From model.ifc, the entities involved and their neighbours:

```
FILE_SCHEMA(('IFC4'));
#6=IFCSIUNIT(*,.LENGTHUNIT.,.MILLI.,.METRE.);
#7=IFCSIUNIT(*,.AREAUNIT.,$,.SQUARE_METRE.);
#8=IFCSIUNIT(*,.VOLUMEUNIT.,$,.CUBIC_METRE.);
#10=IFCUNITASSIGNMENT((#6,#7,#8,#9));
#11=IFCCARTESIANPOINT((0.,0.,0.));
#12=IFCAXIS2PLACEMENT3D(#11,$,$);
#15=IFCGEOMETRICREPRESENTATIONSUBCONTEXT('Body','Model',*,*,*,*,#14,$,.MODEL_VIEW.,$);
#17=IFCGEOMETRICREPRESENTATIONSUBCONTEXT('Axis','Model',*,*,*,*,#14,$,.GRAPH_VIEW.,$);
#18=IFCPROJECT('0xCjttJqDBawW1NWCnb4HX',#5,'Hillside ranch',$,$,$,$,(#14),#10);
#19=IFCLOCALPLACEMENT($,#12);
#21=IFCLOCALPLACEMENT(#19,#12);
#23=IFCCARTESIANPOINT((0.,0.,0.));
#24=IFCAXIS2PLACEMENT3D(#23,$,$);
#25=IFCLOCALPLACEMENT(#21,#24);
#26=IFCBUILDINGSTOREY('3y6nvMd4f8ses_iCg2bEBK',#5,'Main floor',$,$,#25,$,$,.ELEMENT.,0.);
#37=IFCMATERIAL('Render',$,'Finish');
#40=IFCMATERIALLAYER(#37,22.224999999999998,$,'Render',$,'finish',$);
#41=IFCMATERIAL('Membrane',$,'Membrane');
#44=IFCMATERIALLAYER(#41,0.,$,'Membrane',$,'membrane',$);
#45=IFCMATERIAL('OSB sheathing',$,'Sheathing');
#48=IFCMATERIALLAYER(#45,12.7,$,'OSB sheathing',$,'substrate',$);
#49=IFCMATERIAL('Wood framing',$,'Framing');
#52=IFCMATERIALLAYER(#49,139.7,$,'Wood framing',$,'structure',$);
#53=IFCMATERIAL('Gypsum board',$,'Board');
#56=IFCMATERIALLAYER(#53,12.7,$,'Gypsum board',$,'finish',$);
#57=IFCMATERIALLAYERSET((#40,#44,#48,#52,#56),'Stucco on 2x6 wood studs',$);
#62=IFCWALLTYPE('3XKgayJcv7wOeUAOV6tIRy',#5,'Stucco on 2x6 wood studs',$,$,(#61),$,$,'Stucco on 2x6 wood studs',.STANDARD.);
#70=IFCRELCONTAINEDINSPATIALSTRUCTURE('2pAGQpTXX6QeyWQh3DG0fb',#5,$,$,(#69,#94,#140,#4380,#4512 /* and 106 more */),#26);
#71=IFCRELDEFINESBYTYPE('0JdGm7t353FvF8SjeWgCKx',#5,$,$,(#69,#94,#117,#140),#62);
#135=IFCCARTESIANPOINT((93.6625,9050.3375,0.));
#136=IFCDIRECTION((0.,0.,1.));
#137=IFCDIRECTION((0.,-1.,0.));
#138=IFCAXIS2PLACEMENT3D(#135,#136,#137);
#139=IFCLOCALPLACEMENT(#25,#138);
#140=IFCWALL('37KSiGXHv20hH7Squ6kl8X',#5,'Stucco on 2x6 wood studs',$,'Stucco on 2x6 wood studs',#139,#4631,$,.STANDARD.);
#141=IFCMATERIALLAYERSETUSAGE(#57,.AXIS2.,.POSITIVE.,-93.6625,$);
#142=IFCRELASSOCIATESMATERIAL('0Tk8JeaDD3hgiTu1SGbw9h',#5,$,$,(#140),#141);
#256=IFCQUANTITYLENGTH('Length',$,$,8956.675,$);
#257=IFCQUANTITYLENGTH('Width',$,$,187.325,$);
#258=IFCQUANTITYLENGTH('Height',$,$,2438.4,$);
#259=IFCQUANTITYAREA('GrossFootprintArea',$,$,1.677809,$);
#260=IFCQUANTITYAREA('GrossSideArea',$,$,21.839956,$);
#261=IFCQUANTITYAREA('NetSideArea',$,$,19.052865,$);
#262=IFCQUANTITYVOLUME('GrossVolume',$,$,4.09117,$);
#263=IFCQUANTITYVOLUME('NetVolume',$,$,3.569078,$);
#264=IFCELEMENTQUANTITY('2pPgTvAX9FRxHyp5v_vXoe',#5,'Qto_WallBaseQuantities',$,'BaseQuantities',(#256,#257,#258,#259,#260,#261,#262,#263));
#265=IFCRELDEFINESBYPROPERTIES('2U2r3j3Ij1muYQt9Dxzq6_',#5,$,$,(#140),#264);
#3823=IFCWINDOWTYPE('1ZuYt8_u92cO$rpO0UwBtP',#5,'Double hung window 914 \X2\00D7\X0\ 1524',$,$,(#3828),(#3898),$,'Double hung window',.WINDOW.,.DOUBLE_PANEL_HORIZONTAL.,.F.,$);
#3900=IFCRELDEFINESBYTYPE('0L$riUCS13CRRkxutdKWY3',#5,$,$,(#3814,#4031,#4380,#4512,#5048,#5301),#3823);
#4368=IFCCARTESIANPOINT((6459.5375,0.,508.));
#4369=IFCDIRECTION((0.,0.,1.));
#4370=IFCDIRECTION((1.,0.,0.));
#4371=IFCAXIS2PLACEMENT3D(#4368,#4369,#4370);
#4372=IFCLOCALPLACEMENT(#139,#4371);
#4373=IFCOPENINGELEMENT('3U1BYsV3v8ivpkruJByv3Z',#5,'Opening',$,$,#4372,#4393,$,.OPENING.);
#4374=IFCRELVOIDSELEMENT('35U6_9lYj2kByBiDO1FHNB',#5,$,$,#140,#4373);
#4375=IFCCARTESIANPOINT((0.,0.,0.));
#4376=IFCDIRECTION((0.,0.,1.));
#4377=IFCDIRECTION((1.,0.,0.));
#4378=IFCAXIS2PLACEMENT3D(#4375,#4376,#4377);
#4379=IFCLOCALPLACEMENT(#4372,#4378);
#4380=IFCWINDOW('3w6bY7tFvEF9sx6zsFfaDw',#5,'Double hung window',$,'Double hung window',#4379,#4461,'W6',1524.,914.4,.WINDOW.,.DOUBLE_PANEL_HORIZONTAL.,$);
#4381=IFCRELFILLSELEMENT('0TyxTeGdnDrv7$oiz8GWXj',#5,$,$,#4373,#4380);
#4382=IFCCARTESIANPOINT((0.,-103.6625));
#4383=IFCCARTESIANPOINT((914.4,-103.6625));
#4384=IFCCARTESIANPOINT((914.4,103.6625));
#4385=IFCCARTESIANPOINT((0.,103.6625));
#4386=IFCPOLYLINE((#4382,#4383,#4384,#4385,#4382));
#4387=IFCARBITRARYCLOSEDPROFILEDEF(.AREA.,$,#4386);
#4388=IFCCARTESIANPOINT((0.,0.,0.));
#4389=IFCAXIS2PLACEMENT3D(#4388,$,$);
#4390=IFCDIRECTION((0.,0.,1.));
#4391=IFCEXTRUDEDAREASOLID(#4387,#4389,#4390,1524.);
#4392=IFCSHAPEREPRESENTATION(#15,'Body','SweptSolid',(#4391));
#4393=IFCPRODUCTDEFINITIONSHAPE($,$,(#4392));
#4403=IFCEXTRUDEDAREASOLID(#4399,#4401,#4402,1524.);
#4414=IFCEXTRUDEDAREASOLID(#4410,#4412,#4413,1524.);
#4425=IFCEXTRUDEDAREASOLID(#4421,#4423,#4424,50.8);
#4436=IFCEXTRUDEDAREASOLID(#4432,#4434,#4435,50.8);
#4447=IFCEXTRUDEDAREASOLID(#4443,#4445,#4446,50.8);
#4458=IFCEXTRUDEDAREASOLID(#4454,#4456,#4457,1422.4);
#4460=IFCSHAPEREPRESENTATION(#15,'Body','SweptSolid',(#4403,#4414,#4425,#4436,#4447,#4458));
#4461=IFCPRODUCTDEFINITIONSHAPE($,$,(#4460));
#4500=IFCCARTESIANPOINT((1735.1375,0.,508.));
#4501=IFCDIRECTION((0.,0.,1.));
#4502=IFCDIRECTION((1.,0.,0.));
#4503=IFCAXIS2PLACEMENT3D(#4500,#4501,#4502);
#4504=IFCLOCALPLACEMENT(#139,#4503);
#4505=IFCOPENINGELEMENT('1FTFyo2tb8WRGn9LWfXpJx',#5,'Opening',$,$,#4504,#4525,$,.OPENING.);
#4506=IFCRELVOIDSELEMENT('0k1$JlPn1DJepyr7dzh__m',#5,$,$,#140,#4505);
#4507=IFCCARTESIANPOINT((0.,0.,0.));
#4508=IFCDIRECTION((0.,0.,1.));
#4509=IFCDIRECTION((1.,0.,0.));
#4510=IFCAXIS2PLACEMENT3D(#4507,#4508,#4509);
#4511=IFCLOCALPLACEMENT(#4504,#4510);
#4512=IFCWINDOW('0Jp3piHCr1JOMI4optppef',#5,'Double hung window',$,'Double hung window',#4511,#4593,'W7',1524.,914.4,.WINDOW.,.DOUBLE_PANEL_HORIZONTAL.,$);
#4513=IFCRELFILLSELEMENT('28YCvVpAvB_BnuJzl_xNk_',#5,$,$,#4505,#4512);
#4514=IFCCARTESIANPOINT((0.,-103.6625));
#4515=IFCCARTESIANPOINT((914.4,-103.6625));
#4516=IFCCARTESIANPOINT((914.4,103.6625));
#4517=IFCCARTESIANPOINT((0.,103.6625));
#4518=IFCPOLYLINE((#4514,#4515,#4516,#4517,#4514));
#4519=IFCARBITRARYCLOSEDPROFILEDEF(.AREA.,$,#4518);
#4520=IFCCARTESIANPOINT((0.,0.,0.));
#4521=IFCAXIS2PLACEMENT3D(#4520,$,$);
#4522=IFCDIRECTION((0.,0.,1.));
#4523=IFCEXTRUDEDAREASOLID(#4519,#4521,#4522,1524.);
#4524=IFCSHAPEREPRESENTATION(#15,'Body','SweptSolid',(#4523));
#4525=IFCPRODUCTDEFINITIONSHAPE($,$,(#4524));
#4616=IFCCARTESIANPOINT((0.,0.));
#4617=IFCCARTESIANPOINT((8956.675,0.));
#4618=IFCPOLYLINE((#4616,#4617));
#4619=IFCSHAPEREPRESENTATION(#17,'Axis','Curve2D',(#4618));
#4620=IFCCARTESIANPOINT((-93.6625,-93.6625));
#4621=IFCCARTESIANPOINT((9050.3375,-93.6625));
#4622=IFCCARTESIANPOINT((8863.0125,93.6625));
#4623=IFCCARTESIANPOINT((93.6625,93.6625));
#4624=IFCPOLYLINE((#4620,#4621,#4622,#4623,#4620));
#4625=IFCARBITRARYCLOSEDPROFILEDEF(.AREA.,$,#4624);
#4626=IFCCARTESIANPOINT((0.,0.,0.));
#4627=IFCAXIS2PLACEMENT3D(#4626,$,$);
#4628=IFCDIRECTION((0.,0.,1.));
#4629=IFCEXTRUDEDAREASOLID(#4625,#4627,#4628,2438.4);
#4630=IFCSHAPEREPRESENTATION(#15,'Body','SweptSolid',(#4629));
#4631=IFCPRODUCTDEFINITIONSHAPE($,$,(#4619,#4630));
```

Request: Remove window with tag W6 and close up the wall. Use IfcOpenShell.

```python
import ifcopenshell
import ifcopenshell.api.feature
import ifcopenshell.api.pset
import ifcopenshell.api.root
import ifcopenshell.geom
import ifcopenshell.util.element
import ifcopenshell.util.shape
import ifcopenshell.util.unit

model = ifcopenshell.open("model.ifc")
area_scale = ifcopenshell.util.unit.calculate_unit_scale(model, "AREAUNIT")
volume_scale = ifcopenshell.util.unit.calculate_unit_scale(model, "VOLUMEUNIT")
settings = ifcopenshell.geom.settings()


def volume(element):
    """Net volume in cubic metres, openings subtracted."""
    shape = ifcopenshell.geom.create_shape(settings, element)
    return ifcopenshell.util.shape.get_volume(shape.geometry)


window = model.by_id(4380)
opening = window.FillsVoids[0].RelatingOpeningElement
wall = opening.VoidsElements[0].RelatingBuildingElement
before = volume(wall)

ifcopenshell.api.root.remove_product(model, product=window)
ifcopenshell.api.feature.remove_feature(model, feature=opening)

after = volume(wall)
thickness = 0.1873  # wall thickness in metres

# Update the wall's stored quantities.
qto = model.by_id(ifcopenshell.util.element.get_pset(wall, "Qto_WallBaseQuantities", should_inherit=False)["id"])
ifcopenshell.api.pset.edit_qto(model, qto=qto, properties={
    "NetSideArea": after / thickness / area_scale,
    "NetVolume": after / volume_scale,
})

print(f"wall volume {before:.3f} -> {after:.3f} m3")

model.write("model_updated.ifc")
```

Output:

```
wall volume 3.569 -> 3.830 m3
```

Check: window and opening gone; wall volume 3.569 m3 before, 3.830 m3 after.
